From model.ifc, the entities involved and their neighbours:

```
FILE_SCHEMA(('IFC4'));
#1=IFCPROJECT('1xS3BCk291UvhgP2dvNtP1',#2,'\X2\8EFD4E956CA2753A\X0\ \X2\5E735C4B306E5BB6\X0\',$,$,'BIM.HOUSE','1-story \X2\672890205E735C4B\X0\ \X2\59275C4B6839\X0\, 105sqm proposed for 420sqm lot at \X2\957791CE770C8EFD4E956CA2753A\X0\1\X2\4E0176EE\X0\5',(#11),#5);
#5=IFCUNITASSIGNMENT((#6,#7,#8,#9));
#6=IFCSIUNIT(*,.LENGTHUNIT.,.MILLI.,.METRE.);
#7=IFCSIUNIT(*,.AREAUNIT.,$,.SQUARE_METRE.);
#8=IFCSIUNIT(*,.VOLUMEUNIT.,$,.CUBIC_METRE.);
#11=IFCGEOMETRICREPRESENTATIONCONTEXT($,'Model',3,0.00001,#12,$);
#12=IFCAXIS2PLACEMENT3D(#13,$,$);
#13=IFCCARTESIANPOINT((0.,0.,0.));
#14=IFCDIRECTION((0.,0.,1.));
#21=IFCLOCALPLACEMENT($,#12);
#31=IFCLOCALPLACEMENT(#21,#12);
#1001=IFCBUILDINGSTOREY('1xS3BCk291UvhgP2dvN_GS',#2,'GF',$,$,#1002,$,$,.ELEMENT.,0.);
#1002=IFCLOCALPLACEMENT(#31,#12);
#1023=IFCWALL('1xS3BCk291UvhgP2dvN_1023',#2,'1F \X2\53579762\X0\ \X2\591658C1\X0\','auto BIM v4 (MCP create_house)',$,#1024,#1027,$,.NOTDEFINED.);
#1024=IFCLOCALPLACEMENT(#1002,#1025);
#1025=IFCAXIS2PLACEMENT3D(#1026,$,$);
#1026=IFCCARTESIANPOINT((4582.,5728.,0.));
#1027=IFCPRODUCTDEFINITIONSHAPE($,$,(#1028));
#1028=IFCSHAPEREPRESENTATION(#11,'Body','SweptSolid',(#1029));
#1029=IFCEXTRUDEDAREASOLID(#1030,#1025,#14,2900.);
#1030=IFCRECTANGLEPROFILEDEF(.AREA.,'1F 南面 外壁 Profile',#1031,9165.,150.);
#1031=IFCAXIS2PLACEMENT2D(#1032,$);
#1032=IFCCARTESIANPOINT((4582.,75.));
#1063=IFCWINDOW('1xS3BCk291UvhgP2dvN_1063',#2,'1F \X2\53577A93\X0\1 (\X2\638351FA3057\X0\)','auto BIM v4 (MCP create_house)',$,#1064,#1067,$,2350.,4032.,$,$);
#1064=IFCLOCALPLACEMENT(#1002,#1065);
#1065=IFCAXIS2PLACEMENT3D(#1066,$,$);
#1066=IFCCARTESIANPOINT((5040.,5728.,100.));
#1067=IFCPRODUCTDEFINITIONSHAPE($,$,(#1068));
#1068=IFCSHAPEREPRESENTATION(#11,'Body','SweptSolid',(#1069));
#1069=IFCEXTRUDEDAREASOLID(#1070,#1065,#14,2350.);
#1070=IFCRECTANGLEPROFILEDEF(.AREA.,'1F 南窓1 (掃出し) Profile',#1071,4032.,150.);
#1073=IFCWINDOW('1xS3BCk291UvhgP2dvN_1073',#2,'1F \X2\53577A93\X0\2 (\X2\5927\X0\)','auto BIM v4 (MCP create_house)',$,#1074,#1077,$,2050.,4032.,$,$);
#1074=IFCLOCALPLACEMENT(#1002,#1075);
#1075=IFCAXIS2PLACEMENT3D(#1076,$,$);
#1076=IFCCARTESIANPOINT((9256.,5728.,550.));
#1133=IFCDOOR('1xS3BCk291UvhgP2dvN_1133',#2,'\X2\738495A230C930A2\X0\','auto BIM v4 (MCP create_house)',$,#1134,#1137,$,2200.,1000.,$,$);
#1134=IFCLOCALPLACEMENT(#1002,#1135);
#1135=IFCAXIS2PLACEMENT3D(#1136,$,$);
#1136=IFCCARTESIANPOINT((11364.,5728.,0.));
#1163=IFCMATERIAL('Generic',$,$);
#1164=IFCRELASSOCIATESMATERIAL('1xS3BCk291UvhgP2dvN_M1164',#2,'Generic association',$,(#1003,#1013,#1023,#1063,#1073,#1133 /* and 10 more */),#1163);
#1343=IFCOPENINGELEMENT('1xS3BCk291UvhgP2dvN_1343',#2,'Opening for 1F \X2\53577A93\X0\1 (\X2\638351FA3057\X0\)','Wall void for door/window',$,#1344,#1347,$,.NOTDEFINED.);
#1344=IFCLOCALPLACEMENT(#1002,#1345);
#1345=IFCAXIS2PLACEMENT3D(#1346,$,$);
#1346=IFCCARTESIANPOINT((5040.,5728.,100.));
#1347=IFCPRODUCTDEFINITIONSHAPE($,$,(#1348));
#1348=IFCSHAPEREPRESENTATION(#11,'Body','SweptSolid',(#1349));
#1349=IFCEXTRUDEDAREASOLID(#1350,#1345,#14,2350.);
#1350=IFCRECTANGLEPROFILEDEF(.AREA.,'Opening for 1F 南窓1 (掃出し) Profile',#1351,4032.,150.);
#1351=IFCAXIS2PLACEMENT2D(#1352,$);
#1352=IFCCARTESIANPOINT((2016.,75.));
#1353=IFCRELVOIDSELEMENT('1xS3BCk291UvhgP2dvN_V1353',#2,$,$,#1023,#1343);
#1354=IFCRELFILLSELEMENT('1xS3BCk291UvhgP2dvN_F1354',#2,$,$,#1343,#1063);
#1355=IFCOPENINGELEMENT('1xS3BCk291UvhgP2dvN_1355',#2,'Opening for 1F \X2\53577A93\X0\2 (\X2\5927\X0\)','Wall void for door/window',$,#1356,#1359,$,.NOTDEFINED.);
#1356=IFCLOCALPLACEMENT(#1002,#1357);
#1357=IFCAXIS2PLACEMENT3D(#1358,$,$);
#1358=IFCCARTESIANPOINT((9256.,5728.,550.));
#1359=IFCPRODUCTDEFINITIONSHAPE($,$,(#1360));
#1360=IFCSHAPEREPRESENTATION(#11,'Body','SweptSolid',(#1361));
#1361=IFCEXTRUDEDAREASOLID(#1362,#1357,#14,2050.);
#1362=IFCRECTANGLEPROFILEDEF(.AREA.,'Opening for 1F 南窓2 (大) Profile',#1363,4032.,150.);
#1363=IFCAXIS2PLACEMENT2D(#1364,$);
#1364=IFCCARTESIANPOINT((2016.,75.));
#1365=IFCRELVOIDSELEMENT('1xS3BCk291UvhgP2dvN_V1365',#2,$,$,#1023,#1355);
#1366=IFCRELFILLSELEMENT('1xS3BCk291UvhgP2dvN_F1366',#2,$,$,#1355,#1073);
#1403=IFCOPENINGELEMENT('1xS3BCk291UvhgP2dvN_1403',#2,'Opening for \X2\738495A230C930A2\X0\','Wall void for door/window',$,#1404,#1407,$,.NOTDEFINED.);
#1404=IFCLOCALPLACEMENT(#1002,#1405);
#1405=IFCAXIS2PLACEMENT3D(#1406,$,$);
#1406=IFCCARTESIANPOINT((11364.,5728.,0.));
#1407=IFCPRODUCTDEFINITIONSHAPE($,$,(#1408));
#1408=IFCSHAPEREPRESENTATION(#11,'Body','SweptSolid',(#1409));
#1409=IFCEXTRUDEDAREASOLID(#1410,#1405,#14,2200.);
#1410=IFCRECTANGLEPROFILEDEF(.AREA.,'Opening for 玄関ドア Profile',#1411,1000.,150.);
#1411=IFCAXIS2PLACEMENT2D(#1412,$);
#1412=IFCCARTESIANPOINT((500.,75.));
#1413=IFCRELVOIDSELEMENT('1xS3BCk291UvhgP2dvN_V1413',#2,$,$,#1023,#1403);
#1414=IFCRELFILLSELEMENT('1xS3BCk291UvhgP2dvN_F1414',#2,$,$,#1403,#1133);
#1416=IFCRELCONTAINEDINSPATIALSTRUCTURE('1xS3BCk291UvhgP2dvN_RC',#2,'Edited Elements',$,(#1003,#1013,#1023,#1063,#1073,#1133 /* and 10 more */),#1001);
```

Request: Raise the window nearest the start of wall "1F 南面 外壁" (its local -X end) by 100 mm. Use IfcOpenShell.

```python
import numpy as np
import ifcopenshell
import ifcopenshell.api.geometry
import ifcopenshell.util.placement
import ifcopenshell.util.unit

model = ifcopenshell.open("model.ifc")
unit_scale = ifcopenshell.util.unit.calculate_unit_scale(model)

window = model.by_guid("1xS3BCk291UvhgP2dvN_1063")
opening = window.FillsVoids[0].RelatingOpeningElement
dz = 100.0

shift = np.array([0.0, 0.0, dz])
# The window is not placed relative to its opening, so move both.
for product in (opening, window):
    matrix = ifcopenshell.util.placement.get_local_placement(product.ObjectPlacement)
    matrix[:3, 3] += shift
    ifcopenshell.api.geometry.edit_object_placement(model, product=product, matrix=matrix, is_si=False)

print(f"moved by {dz * unit_scale:+.3f} m")

model.write("model_edited.ifc")
```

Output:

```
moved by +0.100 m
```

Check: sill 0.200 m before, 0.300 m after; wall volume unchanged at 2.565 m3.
